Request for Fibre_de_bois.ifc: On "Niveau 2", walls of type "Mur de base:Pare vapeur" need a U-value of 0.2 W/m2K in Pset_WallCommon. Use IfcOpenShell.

First a look at what the model holds.

```python
import ifcopenshell
import ifcopenshell.util.element

model = ifcopenshell.open("Fibre_de_bois.ifc")
print(model.schema)
storey = next(s for s in model.by_type("IfcBuildingStorey") if s.Name == "Niveau 2")
walls = [e for e in ifcopenshell.util.element.get_decomposition(storey) if e.is_a("IfcWall")]
seen = {}
for e in walls:
    element_type = ifcopenshell.util.element.get_type(e)
    key = (element_type.Name if element_type != e and element_type else None, ifcopenshell.util.element.get_pset(e, "Pset_WallCommon", "ThermalTransmittance"))
    seen[key] = seen.get(key, 0) + 1
for (name, value), count in sorted(seen.items(), key=str):
    print(count, "x", name, "|", value)
```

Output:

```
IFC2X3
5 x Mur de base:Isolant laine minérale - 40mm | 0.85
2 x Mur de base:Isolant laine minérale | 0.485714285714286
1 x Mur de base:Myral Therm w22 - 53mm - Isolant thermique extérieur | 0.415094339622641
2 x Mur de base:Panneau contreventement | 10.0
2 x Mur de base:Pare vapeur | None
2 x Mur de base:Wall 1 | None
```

```python
import ifcopenshell
import ifcopenshell.api.pset
import ifcopenshell.util.element

model = ifcopenshell.open("Fibre_de_bois.ifc")

storey = next(s for s in model.by_type("IfcBuildingStorey") if s.Name == "Niveau 2")
walls = [e for e in ifcopenshell.util.element.get_decomposition(storey) if e.is_a("IfcWall")]

count = 0
for e in walls:
    element_type = ifcopenshell.util.element.get_type(e)
    if element_type in (None, e) or element_type.Name != "Mur de base:Pare vapeur":
        continue
    # add_pset returns the element's existing set when there is one.
    pset = ifcopenshell.api.pset.add_pset(model, product=e, name="Pset_WallCommon")
    ifcopenshell.api.pset.edit_pset(model, pset=pset, properties={"ThermalTransmittance": 0.2})
    count += 1

print(count, "walls updated")

model.write("Fibre_de_bois-out.ifc")
```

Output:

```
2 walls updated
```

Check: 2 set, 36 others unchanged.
